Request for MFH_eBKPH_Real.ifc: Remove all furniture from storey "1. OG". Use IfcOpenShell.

First a look at what the model holds.

```python
import ifcopenshell
import ifcopenshell.util.element

model = ifcopenshell.open("MFH_eBKPH_Real.ifc")
print(model.schema)
storey = next(s for s in model.by_type("IfcBuildingStorey") if s.Name == "1. OG")
furniture = [e for e in ifcopenshell.util.element.get_decomposition(storey) if e.is_a("IfcFurnishingElement")]
seen = {}
for e in furniture:
    element_type = ifcopenshell.util.element.get_type(e)
    name = element_type.Name if element_type not in (None, e) else None
    seen[name] = seen.get(name, 0) + 1
for name, count in sorted(seen.items(), key=str):
    print(count, "x", name)
```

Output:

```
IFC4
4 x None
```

```python
import ifcopenshell
import ifcopenshell.api.root
import ifcopenshell.util.element

model = ifcopenshell.open("MFH_eBKPH_Real.ifc")

storey = next(s for s in model.by_type("IfcBuildingStorey") if s.Name == "1. OG")
furniture = [e for e in ifcopenshell.util.element.get_decomposition(storey) if e.is_a("IfcFurnishingElement")]

for e in furniture:
    ifcopenshell.api.root.remove_product(model, product=e)
print(len(furniture), "removed")

model.write("MFH_eBKPH_Real_rev.ifc")
```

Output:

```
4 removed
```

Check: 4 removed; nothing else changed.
